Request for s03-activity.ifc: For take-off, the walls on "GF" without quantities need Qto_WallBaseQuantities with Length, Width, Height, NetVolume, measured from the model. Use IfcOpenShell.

First a look at what the model holds.

```python
import ifcopenshell
import ifcopenshell.util.element
import ifcopenshell.util.unit

model = ifcopenshell.open("s03-activity.ifc")
print(model.schema)
for unit_type in ("LENGTHUNIT", "AREAUNIT", "VOLUMEUNIT"):
    print(unit_type, ifcopenshell.util.unit.calculate_unit_scale(model, unit_type))
storey = next(s for s in model.by_type("IfcBuildingStorey") if s.Name == "GF")
walls = [e for e in ifcopenshell.util.element.get_decomposition(storey) if e.is_a("IfcWall")]
for e in sorted(walls, key=lambda e: e.id()):
    print(e.id(), e.is_a(), e.Name, list(ifcopenshell.util.element.get_psets(e, qtos_only=True)), sep=" | ")
```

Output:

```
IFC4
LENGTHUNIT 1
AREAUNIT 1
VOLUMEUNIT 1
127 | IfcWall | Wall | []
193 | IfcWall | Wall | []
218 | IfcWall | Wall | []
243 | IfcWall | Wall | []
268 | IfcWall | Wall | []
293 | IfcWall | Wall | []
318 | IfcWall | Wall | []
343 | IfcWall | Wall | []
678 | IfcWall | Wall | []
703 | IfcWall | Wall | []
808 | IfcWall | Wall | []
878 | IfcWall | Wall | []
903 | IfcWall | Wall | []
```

```python
import ifcopenshell
import ifcopenshell.api.pset
import ifcopenshell.geom
import ifcopenshell.util.element
import ifcopenshell.util.shape
import ifcopenshell.util.unit

model = ifcopenshell.open("s03-activity.ifc")
unit_scale = ifcopenshell.util.unit.calculate_unit_scale(model)
volume_scale = ifcopenshell.util.unit.calculate_unit_scale(model, "VOLUMEUNIT")
settings = ifcopenshell.geom.settings()

storey = next(s for s in model.by_type("IfcBuildingStorey") if s.Name == "GF")
walls = [e for e in ifcopenshell.util.element.get_decomposition(storey) if e.is_a("IfcWall")]

for e in sorted(walls, key=lambda e: e.id()):
    if ifcopenshell.util.element.get_psets(e, qtos_only=True, should_inherit=False):
        continue
    # Geometry comes back in metres, in the element's own axes.
    shape = ifcopenshell.geom.create_shape(settings, e)
    values = {
        "Length": ifcopenshell.util.shape.get_x(shape.geometry) / unit_scale,
        "Width": ifcopenshell.util.shape.get_y(shape.geometry) / unit_scale,
        "Height": ifcopenshell.util.shape.get_z(shape.geometry) / unit_scale,
        "NetVolume": ifcopenshell.util.shape.get_volume(shape.geometry) / volume_scale,
    }
    qto = ifcopenshell.api.pset.add_qto(model, product=e, name="Qto_WallBaseQuantities")
    ifcopenshell.api.pset.edit_qto(model, qto=qto, properties=values)
    print(e.id(), {k: round(v, 3) for k, v in values.items()})

model.write("s03-activity_rev.ifc")
```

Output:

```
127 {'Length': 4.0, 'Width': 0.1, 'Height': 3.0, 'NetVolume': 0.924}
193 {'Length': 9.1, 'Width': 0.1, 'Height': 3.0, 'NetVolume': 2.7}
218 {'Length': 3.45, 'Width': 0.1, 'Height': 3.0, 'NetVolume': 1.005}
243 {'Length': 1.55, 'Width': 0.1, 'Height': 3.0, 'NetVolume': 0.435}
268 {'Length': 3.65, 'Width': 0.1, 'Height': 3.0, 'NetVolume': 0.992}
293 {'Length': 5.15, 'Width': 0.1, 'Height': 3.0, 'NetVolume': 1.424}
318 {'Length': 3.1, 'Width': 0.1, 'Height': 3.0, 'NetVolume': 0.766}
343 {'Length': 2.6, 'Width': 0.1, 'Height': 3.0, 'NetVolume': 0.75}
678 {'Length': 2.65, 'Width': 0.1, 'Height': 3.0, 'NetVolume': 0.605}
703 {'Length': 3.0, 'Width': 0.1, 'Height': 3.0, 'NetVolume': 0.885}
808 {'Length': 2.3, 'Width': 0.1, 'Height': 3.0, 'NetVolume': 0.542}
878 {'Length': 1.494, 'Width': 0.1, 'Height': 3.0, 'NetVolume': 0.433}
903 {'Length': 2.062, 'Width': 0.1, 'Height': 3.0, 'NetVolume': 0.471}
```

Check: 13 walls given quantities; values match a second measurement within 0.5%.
